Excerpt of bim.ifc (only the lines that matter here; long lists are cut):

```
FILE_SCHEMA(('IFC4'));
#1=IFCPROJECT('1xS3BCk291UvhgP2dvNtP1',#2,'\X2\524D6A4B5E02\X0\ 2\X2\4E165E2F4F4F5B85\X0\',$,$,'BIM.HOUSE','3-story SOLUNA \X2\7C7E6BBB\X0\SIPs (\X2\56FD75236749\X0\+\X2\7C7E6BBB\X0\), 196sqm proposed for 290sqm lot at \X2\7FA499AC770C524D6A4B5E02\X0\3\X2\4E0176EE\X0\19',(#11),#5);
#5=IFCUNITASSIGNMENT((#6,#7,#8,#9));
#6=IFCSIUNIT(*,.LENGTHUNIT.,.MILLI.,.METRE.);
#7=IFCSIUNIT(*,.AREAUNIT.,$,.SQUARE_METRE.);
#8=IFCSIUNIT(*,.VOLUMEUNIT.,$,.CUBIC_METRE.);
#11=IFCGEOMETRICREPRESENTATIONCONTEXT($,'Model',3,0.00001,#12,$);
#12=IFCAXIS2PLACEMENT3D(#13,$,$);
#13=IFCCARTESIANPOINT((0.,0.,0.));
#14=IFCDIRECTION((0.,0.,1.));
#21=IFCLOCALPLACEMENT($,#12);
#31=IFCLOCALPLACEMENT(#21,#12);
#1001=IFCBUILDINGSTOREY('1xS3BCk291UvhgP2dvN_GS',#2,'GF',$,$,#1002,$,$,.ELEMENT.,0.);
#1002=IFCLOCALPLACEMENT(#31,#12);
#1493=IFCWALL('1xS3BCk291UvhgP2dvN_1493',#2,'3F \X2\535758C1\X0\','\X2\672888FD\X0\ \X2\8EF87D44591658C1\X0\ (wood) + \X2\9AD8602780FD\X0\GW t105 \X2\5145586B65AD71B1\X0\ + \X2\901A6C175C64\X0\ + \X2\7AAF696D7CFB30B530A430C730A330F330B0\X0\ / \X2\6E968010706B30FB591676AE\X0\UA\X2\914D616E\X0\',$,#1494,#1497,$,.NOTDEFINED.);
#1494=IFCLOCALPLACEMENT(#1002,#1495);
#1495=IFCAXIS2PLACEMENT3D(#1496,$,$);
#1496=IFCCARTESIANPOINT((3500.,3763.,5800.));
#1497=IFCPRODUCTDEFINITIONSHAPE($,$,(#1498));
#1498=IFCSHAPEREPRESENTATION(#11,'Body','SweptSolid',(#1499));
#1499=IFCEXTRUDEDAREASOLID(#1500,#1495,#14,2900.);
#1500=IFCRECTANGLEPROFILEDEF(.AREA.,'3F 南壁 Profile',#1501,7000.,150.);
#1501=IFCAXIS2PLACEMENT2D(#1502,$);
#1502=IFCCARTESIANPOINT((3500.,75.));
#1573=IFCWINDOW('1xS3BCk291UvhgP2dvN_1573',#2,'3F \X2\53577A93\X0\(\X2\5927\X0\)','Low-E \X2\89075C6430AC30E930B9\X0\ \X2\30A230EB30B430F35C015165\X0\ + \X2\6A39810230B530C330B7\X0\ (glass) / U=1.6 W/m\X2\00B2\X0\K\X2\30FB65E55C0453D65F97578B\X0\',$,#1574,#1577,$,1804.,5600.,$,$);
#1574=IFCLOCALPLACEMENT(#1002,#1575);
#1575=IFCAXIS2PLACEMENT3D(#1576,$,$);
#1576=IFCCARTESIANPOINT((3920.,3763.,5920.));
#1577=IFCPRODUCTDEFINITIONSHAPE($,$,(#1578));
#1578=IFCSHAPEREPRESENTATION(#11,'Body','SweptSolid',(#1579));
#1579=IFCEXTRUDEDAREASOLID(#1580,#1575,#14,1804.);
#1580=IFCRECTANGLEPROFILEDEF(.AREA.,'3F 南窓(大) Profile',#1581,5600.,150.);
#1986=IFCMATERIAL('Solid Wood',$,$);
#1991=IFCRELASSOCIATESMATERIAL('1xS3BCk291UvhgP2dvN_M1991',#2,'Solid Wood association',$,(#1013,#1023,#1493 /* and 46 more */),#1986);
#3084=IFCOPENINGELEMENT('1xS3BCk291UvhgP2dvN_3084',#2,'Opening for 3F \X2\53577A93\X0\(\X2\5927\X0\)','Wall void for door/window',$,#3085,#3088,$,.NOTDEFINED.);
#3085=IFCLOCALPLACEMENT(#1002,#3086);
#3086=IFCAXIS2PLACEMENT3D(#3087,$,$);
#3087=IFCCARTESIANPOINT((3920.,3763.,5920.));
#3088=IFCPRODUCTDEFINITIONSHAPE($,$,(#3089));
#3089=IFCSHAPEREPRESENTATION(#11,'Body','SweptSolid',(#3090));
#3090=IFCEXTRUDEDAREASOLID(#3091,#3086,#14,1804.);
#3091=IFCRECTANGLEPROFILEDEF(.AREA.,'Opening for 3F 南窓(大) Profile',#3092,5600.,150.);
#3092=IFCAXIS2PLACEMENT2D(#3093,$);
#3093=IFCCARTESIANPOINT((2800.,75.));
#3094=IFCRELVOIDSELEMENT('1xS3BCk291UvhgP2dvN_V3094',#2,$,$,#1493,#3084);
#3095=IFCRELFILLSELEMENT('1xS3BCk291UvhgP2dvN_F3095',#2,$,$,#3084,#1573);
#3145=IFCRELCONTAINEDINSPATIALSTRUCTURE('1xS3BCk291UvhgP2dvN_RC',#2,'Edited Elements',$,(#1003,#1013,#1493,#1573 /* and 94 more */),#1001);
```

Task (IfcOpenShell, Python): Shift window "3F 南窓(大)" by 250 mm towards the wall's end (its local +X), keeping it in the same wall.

```python
import ifcopenshell
import ifcopenshell.api.geometry
import ifcopenshell.util.placement

model = ifcopenshell.open("bim.ifc")

window = model.by_guid("1xS3BCk291UvhgP2dvN_1573")
opening = window.FillsVoids[0].RelatingOpeningElement
wall = opening.VoidsElements[0].RelatingBuildingElement

wall_matrix = ifcopenshell.util.placement.get_local_placement(wall.ObjectPlacement)
shift = wall_matrix[:3, 0] * 250.0
before = ifcopenshell.util.placement.get_local_placement(window.ObjectPlacement)[:3, 3].copy()

# The window is not placed relative to its opening, so move both.
for product in (opening, window):
    matrix = ifcopenshell.util.placement.get_local_placement(product.ObjectPlacement)
    matrix[:3, 3] += shift
    ifcopenshell.api.geometry.edit_object_placement(model, product=product, matrix=matrix, is_si=False)

after = ifcopenshell.util.placement.get_local_placement(window.ObjectPlacement)[:3, 3]
print("window moved by", (after - before).round(3) + 0.0)

model.write("bim_v2.ifc")
```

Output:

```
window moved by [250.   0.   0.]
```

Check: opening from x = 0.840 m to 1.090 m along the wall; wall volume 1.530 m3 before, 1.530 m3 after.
